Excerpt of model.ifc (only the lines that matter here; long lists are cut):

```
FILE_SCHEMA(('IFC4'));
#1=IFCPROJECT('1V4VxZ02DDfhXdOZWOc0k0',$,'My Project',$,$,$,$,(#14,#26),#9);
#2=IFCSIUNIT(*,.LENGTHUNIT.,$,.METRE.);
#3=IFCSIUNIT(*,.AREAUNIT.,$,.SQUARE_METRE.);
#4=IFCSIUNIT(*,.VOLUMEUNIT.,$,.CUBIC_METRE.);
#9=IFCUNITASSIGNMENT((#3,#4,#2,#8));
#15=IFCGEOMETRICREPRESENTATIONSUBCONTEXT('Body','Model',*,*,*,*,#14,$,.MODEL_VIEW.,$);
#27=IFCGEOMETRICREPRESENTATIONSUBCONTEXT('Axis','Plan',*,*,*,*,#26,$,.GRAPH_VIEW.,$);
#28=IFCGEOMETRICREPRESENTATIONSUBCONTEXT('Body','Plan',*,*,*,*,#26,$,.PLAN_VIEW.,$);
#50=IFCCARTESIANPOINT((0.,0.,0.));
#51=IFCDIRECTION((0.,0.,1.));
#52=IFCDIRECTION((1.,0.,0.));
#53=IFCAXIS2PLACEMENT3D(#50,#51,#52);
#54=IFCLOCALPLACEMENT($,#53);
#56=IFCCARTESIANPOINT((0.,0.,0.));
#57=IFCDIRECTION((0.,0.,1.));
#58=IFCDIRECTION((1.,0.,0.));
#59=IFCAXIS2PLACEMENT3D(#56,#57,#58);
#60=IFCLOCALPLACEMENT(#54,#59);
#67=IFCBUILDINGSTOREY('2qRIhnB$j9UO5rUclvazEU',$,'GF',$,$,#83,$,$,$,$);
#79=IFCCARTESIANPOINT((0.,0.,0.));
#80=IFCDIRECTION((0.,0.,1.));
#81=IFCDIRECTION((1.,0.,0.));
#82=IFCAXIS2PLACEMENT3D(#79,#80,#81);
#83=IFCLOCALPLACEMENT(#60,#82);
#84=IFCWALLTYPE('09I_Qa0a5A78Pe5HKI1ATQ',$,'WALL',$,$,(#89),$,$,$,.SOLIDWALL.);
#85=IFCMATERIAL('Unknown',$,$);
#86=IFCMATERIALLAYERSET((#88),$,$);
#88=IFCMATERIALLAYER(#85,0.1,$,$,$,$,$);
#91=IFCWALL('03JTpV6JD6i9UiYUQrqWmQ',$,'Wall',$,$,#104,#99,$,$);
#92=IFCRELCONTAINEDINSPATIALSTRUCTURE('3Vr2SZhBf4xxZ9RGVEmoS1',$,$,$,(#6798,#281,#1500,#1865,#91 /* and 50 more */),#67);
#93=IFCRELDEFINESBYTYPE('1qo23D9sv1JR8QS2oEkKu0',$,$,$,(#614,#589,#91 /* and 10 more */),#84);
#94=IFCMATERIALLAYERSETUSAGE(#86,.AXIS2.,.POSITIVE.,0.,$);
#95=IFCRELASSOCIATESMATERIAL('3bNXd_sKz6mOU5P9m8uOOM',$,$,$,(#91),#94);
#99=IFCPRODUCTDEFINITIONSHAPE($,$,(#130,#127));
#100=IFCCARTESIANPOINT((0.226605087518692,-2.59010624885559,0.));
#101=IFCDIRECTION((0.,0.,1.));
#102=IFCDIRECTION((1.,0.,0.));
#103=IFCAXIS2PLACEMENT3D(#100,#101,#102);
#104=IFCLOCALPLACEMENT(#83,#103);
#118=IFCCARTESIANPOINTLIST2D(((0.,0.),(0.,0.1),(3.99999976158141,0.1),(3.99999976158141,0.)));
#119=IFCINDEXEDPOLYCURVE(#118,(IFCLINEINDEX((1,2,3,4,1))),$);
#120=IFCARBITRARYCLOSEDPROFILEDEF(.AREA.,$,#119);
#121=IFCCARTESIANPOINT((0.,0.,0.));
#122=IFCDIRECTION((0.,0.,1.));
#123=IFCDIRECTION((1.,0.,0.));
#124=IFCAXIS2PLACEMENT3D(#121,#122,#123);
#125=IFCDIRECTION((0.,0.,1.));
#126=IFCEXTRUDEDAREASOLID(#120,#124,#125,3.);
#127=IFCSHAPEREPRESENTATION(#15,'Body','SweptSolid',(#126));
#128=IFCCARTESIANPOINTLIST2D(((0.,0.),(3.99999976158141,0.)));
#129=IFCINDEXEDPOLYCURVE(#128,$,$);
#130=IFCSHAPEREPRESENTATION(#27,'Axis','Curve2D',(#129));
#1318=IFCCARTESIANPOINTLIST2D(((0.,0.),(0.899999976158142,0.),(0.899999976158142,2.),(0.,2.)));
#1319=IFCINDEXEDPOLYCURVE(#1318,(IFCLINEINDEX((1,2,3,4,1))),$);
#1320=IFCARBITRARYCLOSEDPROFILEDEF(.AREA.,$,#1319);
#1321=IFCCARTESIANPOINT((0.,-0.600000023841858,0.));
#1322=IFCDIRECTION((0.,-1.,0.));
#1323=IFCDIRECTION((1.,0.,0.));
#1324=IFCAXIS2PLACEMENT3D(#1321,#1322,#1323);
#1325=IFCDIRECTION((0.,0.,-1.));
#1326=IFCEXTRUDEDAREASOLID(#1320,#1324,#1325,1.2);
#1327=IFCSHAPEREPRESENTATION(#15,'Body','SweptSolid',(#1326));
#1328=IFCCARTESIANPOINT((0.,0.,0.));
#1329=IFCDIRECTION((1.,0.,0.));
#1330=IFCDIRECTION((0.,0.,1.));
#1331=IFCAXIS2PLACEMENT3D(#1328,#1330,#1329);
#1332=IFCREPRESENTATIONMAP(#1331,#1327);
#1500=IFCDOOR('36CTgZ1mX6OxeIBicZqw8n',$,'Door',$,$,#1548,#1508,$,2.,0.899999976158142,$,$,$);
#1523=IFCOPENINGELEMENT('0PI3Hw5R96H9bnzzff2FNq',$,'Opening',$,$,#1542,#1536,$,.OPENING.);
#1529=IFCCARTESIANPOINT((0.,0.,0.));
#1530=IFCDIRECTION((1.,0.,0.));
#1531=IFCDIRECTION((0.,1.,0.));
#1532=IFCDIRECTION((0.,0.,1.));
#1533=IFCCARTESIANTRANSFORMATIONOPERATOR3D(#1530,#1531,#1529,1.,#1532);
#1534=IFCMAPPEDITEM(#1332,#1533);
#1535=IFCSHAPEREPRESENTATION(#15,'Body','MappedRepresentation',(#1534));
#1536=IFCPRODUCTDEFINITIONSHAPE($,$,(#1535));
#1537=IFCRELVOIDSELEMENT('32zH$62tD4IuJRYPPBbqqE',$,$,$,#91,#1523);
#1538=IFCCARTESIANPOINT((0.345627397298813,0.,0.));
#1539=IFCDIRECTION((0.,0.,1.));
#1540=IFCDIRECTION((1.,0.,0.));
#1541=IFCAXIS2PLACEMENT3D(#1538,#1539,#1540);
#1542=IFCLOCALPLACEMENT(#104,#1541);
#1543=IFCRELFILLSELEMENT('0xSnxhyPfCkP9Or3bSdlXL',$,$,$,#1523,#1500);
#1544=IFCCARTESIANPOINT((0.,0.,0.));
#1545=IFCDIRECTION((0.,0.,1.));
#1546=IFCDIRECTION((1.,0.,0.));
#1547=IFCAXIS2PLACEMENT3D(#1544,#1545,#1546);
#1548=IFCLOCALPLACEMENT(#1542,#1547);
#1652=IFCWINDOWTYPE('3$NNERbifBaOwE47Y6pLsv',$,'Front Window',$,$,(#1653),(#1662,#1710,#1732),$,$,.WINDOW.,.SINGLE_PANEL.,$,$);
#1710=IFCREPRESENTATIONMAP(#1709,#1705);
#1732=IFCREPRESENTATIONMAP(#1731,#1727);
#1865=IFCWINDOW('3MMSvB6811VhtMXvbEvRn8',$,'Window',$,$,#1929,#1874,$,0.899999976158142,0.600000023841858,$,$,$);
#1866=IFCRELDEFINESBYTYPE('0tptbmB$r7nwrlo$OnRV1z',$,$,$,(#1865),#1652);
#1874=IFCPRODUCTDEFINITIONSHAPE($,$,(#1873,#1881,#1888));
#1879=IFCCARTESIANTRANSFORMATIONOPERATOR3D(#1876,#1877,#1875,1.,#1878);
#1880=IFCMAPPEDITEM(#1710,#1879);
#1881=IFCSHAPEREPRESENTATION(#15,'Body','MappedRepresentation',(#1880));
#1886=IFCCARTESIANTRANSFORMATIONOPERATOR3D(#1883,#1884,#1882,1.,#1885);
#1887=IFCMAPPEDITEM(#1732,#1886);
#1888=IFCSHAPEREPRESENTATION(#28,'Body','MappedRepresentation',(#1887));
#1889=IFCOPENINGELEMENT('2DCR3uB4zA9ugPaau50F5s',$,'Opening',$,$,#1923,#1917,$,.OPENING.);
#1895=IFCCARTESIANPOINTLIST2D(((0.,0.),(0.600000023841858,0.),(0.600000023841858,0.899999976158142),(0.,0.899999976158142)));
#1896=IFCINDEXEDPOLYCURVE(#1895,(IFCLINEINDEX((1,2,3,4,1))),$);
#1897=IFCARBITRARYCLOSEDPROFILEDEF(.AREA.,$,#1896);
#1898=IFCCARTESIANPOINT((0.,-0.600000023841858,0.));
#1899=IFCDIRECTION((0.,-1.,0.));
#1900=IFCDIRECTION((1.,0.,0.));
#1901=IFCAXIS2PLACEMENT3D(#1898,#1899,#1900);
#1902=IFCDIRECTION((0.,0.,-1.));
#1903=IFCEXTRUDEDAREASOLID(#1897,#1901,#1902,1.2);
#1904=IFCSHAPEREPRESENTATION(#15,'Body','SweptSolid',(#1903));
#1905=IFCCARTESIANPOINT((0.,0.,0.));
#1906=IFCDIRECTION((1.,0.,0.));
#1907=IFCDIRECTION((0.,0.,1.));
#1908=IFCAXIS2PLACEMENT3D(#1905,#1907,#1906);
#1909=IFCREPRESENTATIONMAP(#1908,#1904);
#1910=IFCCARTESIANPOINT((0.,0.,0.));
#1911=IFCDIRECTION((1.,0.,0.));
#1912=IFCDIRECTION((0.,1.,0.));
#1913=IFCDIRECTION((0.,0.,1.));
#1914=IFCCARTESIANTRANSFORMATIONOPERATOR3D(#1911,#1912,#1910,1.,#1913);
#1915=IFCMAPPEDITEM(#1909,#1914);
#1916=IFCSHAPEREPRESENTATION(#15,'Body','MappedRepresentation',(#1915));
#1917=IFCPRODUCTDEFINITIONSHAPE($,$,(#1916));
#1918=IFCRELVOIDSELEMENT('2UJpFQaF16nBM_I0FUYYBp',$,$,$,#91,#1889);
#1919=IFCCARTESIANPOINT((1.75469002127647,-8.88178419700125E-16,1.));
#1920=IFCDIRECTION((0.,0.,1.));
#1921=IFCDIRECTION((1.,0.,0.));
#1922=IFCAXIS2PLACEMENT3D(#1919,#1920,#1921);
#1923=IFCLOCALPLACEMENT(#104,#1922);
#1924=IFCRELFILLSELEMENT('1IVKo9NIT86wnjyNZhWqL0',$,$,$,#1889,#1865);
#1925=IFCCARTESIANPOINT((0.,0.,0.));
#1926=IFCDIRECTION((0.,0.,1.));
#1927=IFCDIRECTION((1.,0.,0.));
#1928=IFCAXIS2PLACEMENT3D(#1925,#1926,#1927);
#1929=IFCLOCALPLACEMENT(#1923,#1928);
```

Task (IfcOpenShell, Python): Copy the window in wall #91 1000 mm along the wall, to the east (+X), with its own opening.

```python
import ifcopenshell
import ifcopenshell.api.feature
import ifcopenshell.api.geometry
import ifcopenshell.api.root
import ifcopenshell.geom
import ifcopenshell.util.element
import ifcopenshell.util.placement
import ifcopenshell.util.shape
import ifcopenshell.util.unit

model = ifcopenshell.open("model.ifc")
unit_scale = ifcopenshell.util.unit.calculate_unit_scale(model)
settings = ifcopenshell.geom.settings()


def volume(element):
    """Net volume in cubic metres, openings subtracted."""
    shape = ifcopenshell.geom.create_shape(settings, element)
    return ifcopenshell.util.shape.get_volume(shape.geometry)


window = model.by_id(1865)
opening = window.FillsVoids[0].RelatingOpeningElement
wall = opening.VoidsElements[0].RelatingBuildingElement
before = volume(wall)
shift = ifcopenshell.util.placement.get_local_placement(wall.ObjectPlacement)[:3, 0] * 1 / unit_scale

# copy_class copies the void relationship, type, container and properties, but no geometry.
new_opening = ifcopenshell.api.root.copy_class(model, product=opening)
new_opening.Representation = ifcopenshell.util.element.copy_deep(
    model, opening.Representation, exclude=["IfcGeometricRepresentationContext", "IfcRepresentationMap"]
)
new_window = ifcopenshell.api.root.copy_class(model, product=window)
new_window.Representation = ifcopenshell.util.element.copy_deep(
    model, window.Representation, exclude=["IfcGeometricRepresentationContext", "IfcRepresentationMap"]
)
ifcopenshell.api.feature.add_filling(model, opening=new_opening, element=new_window)

for old, new in ((opening, new_opening), (window, new_window)):
    matrix = ifcopenshell.util.placement.get_local_placement(old.ObjectPlacement)
    matrix[:3, 3] += shift
    ifcopenshell.api.geometry.edit_object_placement(model, product=new, matrix=matrix, is_si=False)

after = volume(wall)

print(f"wall volume {before:.3f} -> {after:.3f} m3")

model.write("model_v2.ifc")
```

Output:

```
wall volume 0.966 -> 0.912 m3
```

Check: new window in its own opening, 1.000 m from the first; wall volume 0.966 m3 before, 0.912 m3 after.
